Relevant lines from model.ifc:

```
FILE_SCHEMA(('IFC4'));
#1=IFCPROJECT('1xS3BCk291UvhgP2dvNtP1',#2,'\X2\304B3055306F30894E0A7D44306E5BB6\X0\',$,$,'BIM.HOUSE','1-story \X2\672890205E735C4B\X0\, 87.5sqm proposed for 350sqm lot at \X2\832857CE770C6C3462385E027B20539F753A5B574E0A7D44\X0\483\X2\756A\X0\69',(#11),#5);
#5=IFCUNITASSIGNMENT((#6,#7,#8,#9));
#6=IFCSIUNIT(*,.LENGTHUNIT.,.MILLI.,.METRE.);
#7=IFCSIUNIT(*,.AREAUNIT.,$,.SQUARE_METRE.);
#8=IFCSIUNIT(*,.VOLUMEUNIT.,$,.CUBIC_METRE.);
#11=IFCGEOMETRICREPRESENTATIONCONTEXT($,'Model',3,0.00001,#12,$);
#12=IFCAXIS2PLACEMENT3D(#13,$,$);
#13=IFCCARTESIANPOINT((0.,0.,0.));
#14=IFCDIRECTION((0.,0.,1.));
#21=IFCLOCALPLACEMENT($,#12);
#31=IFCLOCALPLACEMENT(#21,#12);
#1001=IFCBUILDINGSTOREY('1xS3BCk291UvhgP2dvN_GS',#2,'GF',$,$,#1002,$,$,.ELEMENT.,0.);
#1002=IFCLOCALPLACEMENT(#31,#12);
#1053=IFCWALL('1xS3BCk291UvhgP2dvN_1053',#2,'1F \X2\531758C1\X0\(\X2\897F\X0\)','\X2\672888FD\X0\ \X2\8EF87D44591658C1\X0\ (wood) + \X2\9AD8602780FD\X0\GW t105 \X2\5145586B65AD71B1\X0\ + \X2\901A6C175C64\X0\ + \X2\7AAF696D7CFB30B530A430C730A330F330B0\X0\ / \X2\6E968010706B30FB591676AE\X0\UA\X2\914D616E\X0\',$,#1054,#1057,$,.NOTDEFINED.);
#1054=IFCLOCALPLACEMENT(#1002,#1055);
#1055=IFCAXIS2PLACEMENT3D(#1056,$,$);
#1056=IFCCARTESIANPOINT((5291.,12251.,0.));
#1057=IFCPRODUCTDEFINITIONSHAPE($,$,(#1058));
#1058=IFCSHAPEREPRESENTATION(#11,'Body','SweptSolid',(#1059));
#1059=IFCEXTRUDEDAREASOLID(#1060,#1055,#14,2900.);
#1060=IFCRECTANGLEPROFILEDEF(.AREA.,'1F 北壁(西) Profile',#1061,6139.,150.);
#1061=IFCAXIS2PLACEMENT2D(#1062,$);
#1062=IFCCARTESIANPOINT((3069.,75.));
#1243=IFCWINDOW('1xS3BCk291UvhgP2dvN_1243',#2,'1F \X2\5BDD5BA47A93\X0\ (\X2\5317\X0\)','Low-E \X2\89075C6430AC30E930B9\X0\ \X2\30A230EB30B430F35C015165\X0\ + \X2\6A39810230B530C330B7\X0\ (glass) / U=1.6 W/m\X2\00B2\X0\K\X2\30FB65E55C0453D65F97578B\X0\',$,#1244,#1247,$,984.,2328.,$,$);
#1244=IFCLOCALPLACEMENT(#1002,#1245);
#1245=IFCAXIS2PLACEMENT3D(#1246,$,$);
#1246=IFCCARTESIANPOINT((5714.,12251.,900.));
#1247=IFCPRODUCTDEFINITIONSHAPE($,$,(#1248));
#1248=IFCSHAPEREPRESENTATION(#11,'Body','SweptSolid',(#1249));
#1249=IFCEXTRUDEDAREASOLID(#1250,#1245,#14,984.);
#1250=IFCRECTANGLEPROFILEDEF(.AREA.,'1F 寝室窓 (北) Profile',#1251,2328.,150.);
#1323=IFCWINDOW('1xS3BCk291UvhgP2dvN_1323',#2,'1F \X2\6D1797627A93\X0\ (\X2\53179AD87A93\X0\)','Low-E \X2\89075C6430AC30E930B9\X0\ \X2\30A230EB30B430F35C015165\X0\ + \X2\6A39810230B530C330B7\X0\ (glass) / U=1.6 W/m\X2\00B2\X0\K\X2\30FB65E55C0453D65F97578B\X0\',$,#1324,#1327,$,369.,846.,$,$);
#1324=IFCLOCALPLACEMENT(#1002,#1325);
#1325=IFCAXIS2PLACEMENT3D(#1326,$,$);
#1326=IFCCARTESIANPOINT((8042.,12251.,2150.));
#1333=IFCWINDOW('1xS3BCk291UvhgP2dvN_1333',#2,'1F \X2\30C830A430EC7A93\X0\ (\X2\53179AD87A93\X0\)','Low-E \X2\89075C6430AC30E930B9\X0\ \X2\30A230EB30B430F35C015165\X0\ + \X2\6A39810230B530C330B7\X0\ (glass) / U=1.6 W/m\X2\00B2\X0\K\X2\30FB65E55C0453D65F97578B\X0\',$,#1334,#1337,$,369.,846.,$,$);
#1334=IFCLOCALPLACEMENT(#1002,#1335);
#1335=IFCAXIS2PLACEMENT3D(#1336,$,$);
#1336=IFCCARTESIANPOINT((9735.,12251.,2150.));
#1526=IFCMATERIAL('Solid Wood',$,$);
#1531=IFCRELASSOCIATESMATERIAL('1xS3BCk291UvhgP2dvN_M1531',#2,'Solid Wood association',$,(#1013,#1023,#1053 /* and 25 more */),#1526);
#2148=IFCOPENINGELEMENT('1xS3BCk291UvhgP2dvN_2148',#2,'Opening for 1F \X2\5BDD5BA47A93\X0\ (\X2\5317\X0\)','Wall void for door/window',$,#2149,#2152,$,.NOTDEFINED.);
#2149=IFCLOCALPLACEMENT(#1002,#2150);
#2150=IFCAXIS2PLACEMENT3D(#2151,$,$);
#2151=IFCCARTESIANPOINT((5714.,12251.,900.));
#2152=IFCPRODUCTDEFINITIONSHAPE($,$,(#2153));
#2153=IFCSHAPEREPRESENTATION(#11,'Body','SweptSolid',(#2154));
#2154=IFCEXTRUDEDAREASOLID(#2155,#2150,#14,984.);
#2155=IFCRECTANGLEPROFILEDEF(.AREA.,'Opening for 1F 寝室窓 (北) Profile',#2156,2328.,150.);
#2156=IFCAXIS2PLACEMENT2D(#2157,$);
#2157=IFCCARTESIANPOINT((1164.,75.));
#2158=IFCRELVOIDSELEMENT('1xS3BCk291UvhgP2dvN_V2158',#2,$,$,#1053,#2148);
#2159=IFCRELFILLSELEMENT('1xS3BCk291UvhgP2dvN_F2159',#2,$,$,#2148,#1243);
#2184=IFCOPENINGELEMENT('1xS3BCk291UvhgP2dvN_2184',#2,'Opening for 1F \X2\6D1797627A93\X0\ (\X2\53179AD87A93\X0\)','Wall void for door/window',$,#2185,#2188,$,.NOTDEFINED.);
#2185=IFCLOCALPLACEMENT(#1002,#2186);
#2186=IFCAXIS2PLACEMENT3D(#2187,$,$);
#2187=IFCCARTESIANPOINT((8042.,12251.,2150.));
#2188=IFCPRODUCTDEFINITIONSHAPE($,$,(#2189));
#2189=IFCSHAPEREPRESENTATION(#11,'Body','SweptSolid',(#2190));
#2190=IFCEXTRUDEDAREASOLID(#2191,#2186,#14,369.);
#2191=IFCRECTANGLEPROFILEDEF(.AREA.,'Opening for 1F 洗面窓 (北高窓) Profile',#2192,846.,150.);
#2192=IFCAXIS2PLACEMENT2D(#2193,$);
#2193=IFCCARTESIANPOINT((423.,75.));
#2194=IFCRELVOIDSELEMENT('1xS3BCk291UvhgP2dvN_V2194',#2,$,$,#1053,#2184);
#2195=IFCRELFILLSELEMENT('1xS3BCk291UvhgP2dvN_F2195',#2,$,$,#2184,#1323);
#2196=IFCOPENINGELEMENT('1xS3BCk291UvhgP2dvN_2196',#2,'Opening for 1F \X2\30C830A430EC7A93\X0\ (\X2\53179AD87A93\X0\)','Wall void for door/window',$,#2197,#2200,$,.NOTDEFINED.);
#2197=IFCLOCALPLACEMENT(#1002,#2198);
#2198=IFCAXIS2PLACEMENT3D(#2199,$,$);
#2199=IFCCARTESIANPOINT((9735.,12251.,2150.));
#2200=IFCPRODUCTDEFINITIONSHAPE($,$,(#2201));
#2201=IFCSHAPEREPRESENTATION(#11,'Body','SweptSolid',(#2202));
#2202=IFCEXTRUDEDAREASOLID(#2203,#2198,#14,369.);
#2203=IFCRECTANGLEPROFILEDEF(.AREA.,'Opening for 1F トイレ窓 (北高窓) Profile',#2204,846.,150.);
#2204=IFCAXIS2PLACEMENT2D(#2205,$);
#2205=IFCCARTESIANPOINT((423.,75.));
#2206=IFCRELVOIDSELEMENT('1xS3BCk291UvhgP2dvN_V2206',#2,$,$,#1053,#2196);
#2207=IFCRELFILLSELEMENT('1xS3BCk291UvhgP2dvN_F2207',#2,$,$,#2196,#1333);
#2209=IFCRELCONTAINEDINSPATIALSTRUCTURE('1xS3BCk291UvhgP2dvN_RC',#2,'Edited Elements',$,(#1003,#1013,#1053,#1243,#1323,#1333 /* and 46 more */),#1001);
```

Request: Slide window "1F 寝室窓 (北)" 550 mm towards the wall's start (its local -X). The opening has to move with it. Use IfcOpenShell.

```python
import ifcopenshell
import ifcopenshell.api.geometry
import ifcopenshell.util.placement

model = ifcopenshell.open("model.ifc")

window = model.by_guid("1xS3BCk291UvhgP2dvN_1243")
opening = window.FillsVoids[0].RelatingOpeningElement
wall = opening.VoidsElements[0].RelatingBuildingElement

wall_matrix = ifcopenshell.util.placement.get_local_placement(wall.ObjectPlacement)
shift = wall_matrix[:3, 0] * -550.0
before = ifcopenshell.util.placement.get_local_placement(window.ObjectPlacement)[:3, 3].copy()

# The window is not placed relative to its opening, so move both.
for product in (opening, window):
    matrix = ifcopenshell.util.placement.get_local_placement(product.ObjectPlacement)
    matrix[:3, 3] += shift
    ifcopenshell.api.geometry.edit_object_placement(model, product=product, matrix=matrix, is_si=False)

after = ifcopenshell.util.placement.get_local_placement(window.ObjectPlacement)[:3, 3]
print("window moved by", (after - before).round(3) + 0.0)

model.write("model_rev.ifc")
```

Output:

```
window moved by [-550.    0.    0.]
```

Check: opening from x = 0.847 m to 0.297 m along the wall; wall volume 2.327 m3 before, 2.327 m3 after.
